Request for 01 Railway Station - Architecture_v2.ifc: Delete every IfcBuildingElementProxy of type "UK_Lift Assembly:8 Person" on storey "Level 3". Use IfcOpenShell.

First a look at what the model holds.

```python
import ifcopenshell
import ifcopenshell.util.element

model = ifcopenshell.open("01 Railway Station - Architecture_v2.ifc")
print(model.schema)
storey = next(s for s in model.by_type("IfcBuildingStorey") if s.Name == "Level 3")
proxies = [e for e in ifcopenshell.util.element.get_decomposition(storey) if e.is_a("IfcBuildingElementProxy")]
seen = {}
for e in proxies:
    element_type = ifcopenshell.util.element.get_type(e)
    name = element_type.Name if element_type not in (None, e) else None
    seen[name] = seen.get(name, 0) + 1
for name, count in sorted(seen.items(), key=str):
    print(count, "x", name)
```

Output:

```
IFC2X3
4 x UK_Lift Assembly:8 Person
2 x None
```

```python
import ifcopenshell
import ifcopenshell.api.root
import ifcopenshell.util.element

model = ifcopenshell.open("01 Railway Station - Architecture_v2.ifc")

storey = next(s for s in model.by_type("IfcBuildingStorey") if s.Name == "Level 3")
proxies = [e for e in ifcopenshell.util.element.get_decomposition(storey) if e.is_a("IfcBuildingElementProxy")]
targets = [e for e in proxies if (t := ifcopenshell.util.element.get_type(e)) not in (None, e) and t.Name == "UK_Lift Assembly:8 Person"]

for e in targets:
    ifcopenshell.api.root.remove_product(model, product=e)
print(len(targets), "removed")

model.write("01 Railway Station - Architecture_v2_rev.ifc")
```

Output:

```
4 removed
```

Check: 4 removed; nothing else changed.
